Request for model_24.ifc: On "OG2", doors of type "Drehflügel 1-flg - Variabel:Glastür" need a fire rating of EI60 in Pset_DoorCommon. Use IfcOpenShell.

First a look at what the model holds.

```python
import ifcopenshell
import ifcopenshell.util.element

model = ifcopenshell.open("model_24.ifc")
print(model.schema)
storey = next(s for s in model.by_type("IfcBuildingStorey") if s.Name == "OG2")
doors = [e for e in ifcopenshell.util.element.get_decomposition(storey) if e.is_a("IfcDoor")]
seen = {}
for e in doors:
    element_type = ifcopenshell.util.element.get_type(e)
    key = (element_type.Name if element_type != e and element_type else None, ifcopenshell.util.element.get_pset(e, "Pset_DoorCommon", "FireRating"))
    seen[key] = seen.get(key, 0) + 1
for (name, value), count in sorted(seen.items(), key=str):
    print(count, "x", name, "|", value)
```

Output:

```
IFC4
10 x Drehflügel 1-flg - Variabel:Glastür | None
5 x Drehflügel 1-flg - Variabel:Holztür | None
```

```python
import ifcopenshell
import ifcopenshell.api.pset
import ifcopenshell.util.element

model = ifcopenshell.open("model_24.ifc")

storey = next(s for s in model.by_type("IfcBuildingStorey") if s.Name == "OG2")
doors = [e for e in ifcopenshell.util.element.get_decomposition(storey) if e.is_a("IfcDoor")]

count = 0
for e in doors:
    element_type = ifcopenshell.util.element.get_type(e)
    if element_type in (None, e) or element_type.Name != "Drehflügel 1-flg - Variabel:Glastür":
        continue
    # add_pset returns the element's existing set when there is one.
    pset = ifcopenshell.api.pset.add_pset(model, product=e, name="Pset_DoorCommon")
    ifcopenshell.api.pset.edit_pset(model, pset=pset, properties={"FireRating": "EI60"})
    count += 1

print(count, "doors updated")

model.write("model_24_rev.ifc")
```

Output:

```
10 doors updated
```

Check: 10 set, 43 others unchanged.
